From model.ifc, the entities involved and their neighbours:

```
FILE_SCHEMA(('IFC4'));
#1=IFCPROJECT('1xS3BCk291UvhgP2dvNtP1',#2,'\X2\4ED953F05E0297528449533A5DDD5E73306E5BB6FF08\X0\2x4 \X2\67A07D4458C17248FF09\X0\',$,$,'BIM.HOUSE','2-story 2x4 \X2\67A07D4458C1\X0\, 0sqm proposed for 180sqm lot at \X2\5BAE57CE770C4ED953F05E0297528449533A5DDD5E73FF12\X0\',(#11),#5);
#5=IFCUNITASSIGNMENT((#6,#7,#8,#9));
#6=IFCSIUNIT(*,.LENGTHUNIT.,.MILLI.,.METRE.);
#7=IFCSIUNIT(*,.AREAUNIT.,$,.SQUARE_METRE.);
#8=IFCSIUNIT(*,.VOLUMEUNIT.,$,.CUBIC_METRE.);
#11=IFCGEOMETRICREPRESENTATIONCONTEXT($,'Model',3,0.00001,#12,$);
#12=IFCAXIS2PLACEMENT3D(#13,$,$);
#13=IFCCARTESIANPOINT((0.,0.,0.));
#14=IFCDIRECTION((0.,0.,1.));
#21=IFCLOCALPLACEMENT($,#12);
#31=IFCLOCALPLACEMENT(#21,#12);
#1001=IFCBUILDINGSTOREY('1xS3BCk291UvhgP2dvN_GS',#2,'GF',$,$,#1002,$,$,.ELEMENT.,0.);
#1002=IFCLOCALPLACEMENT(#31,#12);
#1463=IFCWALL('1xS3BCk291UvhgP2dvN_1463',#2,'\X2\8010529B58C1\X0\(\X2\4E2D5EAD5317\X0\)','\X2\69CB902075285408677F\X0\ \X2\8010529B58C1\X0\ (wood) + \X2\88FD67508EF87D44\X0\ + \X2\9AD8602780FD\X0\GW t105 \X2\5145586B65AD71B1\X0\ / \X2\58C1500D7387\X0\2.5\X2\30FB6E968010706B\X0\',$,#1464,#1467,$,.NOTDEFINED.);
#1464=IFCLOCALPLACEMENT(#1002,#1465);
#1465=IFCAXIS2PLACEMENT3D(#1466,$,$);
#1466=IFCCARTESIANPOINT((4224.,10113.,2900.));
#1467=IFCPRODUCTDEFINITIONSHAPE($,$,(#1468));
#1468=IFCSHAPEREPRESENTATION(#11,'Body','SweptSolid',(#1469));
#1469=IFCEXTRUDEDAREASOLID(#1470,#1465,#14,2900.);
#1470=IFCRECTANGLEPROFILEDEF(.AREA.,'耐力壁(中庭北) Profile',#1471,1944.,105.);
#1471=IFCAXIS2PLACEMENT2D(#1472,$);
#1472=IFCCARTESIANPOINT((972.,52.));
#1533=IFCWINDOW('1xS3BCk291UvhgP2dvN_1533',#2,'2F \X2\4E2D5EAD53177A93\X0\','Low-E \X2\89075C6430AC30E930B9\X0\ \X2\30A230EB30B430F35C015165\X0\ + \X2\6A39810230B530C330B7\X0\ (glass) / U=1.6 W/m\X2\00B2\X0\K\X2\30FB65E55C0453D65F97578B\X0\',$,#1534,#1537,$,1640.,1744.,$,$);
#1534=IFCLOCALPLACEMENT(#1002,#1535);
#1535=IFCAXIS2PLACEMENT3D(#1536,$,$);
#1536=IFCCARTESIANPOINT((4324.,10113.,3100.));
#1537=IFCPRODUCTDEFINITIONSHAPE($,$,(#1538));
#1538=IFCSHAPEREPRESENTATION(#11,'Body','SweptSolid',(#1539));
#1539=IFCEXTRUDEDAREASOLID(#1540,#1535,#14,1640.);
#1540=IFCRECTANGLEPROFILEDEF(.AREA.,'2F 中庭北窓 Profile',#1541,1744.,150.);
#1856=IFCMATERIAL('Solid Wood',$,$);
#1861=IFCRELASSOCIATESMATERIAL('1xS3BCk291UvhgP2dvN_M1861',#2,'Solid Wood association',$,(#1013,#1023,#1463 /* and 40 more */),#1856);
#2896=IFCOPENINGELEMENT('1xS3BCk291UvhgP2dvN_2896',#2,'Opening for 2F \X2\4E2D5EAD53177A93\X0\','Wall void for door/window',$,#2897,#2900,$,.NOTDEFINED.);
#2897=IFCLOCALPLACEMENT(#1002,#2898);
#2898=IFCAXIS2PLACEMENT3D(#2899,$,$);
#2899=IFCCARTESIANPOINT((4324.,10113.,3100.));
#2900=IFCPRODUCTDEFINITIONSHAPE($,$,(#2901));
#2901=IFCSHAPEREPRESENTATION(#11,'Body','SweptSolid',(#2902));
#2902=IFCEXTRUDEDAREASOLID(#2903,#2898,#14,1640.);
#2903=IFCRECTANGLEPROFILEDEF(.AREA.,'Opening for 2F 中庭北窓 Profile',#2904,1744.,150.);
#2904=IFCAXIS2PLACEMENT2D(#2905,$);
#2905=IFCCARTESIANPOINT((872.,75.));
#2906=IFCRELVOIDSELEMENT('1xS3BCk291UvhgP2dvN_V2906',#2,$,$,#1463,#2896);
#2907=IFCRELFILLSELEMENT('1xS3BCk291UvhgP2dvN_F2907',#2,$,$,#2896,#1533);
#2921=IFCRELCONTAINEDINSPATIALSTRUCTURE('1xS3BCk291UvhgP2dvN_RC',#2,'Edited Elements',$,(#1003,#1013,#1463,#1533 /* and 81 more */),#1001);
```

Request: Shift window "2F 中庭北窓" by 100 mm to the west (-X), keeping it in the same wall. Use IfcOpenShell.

```python
import ifcopenshell
import ifcopenshell.api.geometry
import ifcopenshell.util.placement
import ifcopenshell.util.unit

model = ifcopenshell.open("model.ifc")
unit_scale = ifcopenshell.util.unit.calculate_unit_scale(model)

window = model.by_guid("1xS3BCk291UvhgP2dvN_1533")
opening = window.FillsVoids[0].RelatingOpeningElement
wall = opening.VoidsElements[0].RelatingBuildingElement

wall_matrix = ifcopenshell.util.placement.get_local_placement(wall.ObjectPlacement)
shift = wall_matrix[:3, 0] * -0.1 / unit_scale
before = ifcopenshell.util.placement.get_local_placement(window.ObjectPlacement)[:3, 3].copy()

# The window is not placed relative to its opening, so move both.
for product in (opening, window):
    matrix = ifcopenshell.util.placement.get_local_placement(product.ObjectPlacement)
    matrix[:3, 3] += shift
    ifcopenshell.api.geometry.edit_object_placement(model, product=product, matrix=matrix, is_si=False)

after = ifcopenshell.util.placement.get_local_placement(window.ObjectPlacement)[:3, 3]
print("window moved by", (after - before).round(3) + 0.0)

model.write("model_updated.ifc")
```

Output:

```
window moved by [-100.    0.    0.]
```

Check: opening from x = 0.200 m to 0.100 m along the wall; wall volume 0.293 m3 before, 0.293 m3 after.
